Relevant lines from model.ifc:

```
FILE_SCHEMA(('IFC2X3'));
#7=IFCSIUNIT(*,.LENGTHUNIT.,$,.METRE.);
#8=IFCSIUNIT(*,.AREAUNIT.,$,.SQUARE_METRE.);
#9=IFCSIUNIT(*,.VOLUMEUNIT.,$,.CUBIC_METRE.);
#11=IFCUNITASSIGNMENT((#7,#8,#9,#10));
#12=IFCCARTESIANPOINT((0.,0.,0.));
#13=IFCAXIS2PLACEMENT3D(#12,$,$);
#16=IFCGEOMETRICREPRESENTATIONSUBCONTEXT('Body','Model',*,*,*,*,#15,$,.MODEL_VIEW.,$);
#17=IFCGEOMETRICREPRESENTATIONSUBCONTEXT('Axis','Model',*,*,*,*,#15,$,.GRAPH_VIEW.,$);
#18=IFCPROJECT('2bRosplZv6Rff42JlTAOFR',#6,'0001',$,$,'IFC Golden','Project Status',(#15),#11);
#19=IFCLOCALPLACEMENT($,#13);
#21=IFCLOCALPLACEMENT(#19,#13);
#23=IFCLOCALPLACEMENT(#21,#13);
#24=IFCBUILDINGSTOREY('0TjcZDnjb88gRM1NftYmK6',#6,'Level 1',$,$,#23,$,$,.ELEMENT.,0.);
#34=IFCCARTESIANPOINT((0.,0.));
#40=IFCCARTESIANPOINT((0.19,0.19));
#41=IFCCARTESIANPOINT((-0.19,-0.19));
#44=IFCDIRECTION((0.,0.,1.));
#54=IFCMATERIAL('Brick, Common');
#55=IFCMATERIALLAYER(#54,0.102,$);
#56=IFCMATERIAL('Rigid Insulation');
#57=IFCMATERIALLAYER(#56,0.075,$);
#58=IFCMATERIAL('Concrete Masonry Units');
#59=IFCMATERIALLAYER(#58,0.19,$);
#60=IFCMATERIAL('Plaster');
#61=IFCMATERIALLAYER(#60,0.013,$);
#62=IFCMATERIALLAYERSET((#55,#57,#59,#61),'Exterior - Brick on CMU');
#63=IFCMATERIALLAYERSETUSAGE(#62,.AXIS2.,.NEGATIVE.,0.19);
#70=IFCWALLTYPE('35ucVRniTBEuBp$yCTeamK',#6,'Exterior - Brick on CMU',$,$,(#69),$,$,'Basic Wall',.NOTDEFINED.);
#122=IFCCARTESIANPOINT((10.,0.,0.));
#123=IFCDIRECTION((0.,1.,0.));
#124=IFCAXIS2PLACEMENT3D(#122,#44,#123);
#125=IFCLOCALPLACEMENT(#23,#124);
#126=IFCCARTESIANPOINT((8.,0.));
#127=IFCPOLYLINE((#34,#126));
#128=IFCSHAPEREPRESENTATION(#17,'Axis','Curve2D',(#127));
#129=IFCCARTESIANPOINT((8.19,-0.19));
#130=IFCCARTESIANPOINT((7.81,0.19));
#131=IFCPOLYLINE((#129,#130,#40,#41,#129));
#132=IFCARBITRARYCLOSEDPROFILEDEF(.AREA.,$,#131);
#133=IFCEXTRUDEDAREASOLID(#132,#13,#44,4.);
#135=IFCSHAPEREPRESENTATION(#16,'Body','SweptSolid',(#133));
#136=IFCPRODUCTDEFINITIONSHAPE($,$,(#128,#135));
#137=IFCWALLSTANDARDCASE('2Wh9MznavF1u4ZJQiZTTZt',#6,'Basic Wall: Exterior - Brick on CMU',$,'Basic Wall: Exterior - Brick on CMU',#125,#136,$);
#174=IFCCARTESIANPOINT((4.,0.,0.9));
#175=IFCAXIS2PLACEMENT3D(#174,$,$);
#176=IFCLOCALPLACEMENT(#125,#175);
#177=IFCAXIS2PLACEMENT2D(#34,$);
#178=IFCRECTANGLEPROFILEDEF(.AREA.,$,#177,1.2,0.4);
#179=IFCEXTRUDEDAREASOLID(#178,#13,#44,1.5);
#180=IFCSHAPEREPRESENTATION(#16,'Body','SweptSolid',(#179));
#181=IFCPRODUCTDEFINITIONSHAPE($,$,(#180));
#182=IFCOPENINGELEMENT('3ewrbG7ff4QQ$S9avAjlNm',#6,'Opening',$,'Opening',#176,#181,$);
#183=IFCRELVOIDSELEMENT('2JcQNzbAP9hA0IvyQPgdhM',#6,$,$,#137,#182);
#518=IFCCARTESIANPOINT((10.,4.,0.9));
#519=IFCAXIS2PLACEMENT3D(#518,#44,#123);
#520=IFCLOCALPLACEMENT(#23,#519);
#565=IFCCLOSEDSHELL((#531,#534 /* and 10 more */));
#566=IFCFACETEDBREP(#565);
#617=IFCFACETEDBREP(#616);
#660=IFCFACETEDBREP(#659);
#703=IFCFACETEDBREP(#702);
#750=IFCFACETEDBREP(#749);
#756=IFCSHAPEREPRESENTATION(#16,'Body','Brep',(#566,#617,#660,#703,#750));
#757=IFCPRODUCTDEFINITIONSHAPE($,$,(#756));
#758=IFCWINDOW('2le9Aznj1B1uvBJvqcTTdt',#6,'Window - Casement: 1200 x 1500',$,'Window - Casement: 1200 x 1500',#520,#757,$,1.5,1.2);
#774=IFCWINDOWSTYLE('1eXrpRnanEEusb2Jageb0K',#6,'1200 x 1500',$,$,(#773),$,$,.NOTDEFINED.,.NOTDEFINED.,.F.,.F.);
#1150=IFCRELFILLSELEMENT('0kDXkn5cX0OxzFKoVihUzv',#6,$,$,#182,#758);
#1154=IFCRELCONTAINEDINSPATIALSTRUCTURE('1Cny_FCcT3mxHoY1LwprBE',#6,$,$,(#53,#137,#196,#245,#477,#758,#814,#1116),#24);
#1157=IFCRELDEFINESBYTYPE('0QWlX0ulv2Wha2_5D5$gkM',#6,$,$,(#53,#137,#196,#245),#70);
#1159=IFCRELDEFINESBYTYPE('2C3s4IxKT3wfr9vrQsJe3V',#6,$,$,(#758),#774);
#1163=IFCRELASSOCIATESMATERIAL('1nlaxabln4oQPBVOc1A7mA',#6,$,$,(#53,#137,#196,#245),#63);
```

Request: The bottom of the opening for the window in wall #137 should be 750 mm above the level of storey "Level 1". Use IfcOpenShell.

```python
import numpy as np
import ifcopenshell
import ifcopenshell.api.geometry
import ifcopenshell.geom
import ifcopenshell.util.element
import ifcopenshell.util.placement
import ifcopenshell.util.shape
import ifcopenshell.util.unit

model = ifcopenshell.open("model.ifc")
unit_scale = ifcopenshell.util.unit.calculate_unit_scale(model)

window = model.by_id(758)
opening = window.FillsVoids[0].RelatingOpeningElement
storey = ifcopenshell.util.element.get_container(window, ifc_class="IfcBuildingStorey")
level = ifcopenshell.util.placement.get_local_placement(storey.ObjectPlacement)[2, 3]

# The opening's origin need not be at the sill, so measure its lowest point.
shape = ifcopenshell.geom.create_shape(ifcopenshell.geom.settings(), opening)
bottom = ifcopenshell.util.shape.get_shape_bottom_elevation(shape, shape.geometry) / unit_scale
dz = level + 0.75 - bottom

shift = np.array([0.0, 0.0, dz])
# The window is not placed relative to its opening, so move both.
for product in (opening, window):
    matrix = ifcopenshell.util.placement.get_local_placement(product.ObjectPlacement)
    matrix[:3, 3] += shift
    ifcopenshell.api.geometry.edit_object_placement(model, product=product, matrix=matrix, is_si=False)

print(f"moved by {dz * unit_scale:+.3f} m")

model.write("model_updated.ifc")
```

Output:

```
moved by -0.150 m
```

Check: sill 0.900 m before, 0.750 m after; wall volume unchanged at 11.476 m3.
